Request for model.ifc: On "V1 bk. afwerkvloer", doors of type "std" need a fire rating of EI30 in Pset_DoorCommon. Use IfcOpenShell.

First a look at what the model holds.

```python
import ifcopenshell
import ifcopenshell.util.element

model = ifcopenshell.open("model.ifc")
print(model.schema)
storey = next(s for s in model.by_type("IfcBuildingStorey") if s.Name == "V1 bk. afwerkvloer")
doors = [e for e in ifcopenshell.util.element.get_decomposition(storey) if e.is_a("IfcDoor")]
seen = {}
for e in doors:
    element_type = ifcopenshell.util.element.get_type(e)
    key = (element_type.Name if element_type != e and element_type else None, ifcopenshell.util.element.get_pset(e, "Pset_DoorCommon", "FireRating"))
    seen[key] = seen.get(key, 0) + 1
for (name, value), count in sorted(seen.items(), key=str):
    print(count, "x", name, "|", value)
```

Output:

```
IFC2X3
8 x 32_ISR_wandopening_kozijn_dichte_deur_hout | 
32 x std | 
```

```python
import ifcopenshell
import ifcopenshell.api.pset
import ifcopenshell.util.element

model = ifcopenshell.open("model.ifc")

storey = next(s for s in model.by_type("IfcBuildingStorey") if s.Name == "V1 bk. afwerkvloer")
doors = [e for e in ifcopenshell.util.element.get_decomposition(storey) if e.is_a("IfcDoor")]

count = 0
for e in doors:
    element_type = ifcopenshell.util.element.get_type(e)
    if element_type in (None, e) or element_type.Name != "std":
        continue
    # add_pset returns the element's existing set when there is one.
    pset = ifcopenshell.api.pset.add_pset(model, product=e, name="Pset_DoorCommon")
    ifcopenshell.api.pset.edit_pset(model, pset=pset, properties={"FireRating": "EI30"})
    count += 1

print(count, "doors updated")

model.write("model-out.ifc")
```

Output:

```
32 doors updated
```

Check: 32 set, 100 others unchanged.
